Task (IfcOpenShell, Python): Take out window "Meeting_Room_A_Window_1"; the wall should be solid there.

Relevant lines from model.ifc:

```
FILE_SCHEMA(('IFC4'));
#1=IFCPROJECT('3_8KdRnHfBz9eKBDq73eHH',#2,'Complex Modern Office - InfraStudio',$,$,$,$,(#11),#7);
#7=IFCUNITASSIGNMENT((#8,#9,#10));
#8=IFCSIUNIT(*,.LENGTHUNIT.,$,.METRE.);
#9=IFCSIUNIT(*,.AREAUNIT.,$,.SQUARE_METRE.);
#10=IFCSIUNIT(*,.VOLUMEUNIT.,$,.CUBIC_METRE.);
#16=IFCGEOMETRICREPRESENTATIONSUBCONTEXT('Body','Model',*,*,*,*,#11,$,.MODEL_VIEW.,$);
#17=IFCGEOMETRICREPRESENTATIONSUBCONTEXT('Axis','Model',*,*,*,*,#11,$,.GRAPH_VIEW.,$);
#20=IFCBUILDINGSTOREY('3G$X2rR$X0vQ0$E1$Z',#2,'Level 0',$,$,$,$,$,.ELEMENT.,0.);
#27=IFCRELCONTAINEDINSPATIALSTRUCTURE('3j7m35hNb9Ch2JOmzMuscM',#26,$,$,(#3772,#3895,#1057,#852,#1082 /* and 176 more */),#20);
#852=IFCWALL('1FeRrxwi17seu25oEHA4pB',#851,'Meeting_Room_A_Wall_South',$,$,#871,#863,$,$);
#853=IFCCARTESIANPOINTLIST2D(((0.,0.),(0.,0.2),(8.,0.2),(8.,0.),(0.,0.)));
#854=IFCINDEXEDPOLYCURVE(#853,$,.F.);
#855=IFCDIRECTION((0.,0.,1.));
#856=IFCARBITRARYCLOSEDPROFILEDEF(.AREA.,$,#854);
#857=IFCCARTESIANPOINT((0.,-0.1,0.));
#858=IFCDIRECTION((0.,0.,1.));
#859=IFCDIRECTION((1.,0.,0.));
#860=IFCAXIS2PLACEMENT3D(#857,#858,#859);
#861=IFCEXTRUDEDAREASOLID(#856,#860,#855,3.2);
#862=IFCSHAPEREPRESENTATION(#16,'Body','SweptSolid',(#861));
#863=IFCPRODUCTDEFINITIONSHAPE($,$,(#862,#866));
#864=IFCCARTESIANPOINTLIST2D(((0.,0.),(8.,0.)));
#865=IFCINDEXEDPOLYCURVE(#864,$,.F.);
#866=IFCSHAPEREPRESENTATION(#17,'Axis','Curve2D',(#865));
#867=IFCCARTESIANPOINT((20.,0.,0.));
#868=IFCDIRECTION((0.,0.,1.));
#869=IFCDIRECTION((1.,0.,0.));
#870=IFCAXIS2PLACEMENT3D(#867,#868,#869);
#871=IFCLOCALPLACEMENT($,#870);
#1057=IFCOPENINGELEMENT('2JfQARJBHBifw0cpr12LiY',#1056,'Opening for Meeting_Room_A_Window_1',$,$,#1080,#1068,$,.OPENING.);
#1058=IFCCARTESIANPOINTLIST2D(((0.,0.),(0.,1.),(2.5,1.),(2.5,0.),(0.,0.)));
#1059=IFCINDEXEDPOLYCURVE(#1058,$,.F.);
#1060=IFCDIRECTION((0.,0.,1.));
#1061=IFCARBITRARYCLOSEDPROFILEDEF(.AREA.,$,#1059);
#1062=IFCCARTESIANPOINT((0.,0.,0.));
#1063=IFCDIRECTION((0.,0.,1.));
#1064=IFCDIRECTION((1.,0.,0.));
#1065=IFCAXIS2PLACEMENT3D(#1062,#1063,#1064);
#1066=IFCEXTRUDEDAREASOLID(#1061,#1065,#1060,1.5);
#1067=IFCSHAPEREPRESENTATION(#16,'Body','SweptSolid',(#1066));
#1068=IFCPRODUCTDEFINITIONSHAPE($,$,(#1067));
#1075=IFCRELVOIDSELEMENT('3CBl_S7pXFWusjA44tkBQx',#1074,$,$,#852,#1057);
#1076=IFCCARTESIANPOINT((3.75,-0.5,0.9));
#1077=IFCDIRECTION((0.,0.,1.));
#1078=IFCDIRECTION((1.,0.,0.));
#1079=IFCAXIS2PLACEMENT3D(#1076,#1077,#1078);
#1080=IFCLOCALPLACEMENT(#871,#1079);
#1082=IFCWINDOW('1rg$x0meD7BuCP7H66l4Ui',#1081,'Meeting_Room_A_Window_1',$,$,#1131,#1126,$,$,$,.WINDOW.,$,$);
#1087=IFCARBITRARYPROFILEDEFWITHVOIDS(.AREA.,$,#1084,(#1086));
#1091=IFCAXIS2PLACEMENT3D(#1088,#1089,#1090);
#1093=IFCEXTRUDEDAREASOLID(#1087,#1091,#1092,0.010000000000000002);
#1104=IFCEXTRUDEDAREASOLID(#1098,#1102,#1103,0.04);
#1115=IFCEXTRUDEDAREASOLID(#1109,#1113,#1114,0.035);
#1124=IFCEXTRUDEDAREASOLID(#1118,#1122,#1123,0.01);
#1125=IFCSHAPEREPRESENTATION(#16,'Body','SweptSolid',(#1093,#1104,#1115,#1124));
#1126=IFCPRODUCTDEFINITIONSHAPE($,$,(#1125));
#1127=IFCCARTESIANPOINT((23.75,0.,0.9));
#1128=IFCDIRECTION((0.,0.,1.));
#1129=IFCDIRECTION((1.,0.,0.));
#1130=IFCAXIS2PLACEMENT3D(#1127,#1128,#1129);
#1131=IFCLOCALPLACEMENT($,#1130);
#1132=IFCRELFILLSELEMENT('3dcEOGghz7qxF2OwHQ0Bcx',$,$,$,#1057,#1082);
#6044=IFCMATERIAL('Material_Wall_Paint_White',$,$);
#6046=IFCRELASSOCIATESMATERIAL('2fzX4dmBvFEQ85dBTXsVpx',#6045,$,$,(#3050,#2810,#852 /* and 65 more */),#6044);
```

```python
import ifcopenshell
import ifcopenshell.api.feature
import ifcopenshell.api.root
import ifcopenshell.geom
import ifcopenshell.util.shape

model = ifcopenshell.open("model.ifc")
settings = ifcopenshell.geom.settings()


def volume(element):
    """Net volume in cubic metres, openings subtracted."""
    shape = ifcopenshell.geom.create_shape(settings, element)
    return ifcopenshell.util.shape.get_volume(shape.geometry)


window = model.by_id(1082)
opening = window.FillsVoids[0].RelatingOpeningElement
wall = opening.VoidsElements[0].RelatingBuildingElement
before = volume(wall)

ifcopenshell.api.root.remove_product(model, product=window)
ifcopenshell.api.feature.remove_feature(model, feature=opening)

after = volume(wall)

print(f"wall volume {before:.3f} -> {after:.3f} m3")

model.write("model-out.ifc")
```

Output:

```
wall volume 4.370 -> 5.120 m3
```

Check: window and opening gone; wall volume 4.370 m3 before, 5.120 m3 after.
